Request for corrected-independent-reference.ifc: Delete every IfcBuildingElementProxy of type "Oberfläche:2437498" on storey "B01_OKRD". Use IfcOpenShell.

First a look at what the model holds.

```python
import ifcopenshell
import ifcopenshell.util.element

model = ifcopenshell.open("corrected-independent-reference.ifc")
print(model.schema)
storey = next(s for s in model.by_type("IfcBuildingStorey") if s.Name == "B01_OKRD")
proxies = [e for e in ifcopenshell.util.element.get_decomposition(storey) if e.is_a("IfcBuildingElementProxy")]
seen = {}
for e in proxies:
    element_type = ifcopenshell.util.element.get_type(e)
    name = element_type.Name if element_type not in (None, e) else None
    seen[name] = seen.get(name, 0) + 1
for name, count in sorted(seen.items(), key=str):
    print(count, "x", name)
```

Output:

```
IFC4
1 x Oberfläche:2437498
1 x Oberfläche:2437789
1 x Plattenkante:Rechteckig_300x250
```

```python
import ifcopenshell
import ifcopenshell.api.root
import ifcopenshell.util.element

model = ifcopenshell.open("corrected-independent-reference.ifc")

storey = next(s for s in model.by_type("IfcBuildingStorey") if s.Name == "B01_OKRD")
proxies = [e for e in ifcopenshell.util.element.get_decomposition(storey) if e.is_a("IfcBuildingElementProxy")]
targets = [e for e in proxies if (t := ifcopenshell.util.element.get_type(e)) not in (None, e) and t.Name == "Oberfläche:2437498"]

for e in targets:
    ifcopenshell.api.root.remove_product(model, product=e)
print(len(targets), "removed")

model.write("corrected-independent-reference_updated.ifc")
```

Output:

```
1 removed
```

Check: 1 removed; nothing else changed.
